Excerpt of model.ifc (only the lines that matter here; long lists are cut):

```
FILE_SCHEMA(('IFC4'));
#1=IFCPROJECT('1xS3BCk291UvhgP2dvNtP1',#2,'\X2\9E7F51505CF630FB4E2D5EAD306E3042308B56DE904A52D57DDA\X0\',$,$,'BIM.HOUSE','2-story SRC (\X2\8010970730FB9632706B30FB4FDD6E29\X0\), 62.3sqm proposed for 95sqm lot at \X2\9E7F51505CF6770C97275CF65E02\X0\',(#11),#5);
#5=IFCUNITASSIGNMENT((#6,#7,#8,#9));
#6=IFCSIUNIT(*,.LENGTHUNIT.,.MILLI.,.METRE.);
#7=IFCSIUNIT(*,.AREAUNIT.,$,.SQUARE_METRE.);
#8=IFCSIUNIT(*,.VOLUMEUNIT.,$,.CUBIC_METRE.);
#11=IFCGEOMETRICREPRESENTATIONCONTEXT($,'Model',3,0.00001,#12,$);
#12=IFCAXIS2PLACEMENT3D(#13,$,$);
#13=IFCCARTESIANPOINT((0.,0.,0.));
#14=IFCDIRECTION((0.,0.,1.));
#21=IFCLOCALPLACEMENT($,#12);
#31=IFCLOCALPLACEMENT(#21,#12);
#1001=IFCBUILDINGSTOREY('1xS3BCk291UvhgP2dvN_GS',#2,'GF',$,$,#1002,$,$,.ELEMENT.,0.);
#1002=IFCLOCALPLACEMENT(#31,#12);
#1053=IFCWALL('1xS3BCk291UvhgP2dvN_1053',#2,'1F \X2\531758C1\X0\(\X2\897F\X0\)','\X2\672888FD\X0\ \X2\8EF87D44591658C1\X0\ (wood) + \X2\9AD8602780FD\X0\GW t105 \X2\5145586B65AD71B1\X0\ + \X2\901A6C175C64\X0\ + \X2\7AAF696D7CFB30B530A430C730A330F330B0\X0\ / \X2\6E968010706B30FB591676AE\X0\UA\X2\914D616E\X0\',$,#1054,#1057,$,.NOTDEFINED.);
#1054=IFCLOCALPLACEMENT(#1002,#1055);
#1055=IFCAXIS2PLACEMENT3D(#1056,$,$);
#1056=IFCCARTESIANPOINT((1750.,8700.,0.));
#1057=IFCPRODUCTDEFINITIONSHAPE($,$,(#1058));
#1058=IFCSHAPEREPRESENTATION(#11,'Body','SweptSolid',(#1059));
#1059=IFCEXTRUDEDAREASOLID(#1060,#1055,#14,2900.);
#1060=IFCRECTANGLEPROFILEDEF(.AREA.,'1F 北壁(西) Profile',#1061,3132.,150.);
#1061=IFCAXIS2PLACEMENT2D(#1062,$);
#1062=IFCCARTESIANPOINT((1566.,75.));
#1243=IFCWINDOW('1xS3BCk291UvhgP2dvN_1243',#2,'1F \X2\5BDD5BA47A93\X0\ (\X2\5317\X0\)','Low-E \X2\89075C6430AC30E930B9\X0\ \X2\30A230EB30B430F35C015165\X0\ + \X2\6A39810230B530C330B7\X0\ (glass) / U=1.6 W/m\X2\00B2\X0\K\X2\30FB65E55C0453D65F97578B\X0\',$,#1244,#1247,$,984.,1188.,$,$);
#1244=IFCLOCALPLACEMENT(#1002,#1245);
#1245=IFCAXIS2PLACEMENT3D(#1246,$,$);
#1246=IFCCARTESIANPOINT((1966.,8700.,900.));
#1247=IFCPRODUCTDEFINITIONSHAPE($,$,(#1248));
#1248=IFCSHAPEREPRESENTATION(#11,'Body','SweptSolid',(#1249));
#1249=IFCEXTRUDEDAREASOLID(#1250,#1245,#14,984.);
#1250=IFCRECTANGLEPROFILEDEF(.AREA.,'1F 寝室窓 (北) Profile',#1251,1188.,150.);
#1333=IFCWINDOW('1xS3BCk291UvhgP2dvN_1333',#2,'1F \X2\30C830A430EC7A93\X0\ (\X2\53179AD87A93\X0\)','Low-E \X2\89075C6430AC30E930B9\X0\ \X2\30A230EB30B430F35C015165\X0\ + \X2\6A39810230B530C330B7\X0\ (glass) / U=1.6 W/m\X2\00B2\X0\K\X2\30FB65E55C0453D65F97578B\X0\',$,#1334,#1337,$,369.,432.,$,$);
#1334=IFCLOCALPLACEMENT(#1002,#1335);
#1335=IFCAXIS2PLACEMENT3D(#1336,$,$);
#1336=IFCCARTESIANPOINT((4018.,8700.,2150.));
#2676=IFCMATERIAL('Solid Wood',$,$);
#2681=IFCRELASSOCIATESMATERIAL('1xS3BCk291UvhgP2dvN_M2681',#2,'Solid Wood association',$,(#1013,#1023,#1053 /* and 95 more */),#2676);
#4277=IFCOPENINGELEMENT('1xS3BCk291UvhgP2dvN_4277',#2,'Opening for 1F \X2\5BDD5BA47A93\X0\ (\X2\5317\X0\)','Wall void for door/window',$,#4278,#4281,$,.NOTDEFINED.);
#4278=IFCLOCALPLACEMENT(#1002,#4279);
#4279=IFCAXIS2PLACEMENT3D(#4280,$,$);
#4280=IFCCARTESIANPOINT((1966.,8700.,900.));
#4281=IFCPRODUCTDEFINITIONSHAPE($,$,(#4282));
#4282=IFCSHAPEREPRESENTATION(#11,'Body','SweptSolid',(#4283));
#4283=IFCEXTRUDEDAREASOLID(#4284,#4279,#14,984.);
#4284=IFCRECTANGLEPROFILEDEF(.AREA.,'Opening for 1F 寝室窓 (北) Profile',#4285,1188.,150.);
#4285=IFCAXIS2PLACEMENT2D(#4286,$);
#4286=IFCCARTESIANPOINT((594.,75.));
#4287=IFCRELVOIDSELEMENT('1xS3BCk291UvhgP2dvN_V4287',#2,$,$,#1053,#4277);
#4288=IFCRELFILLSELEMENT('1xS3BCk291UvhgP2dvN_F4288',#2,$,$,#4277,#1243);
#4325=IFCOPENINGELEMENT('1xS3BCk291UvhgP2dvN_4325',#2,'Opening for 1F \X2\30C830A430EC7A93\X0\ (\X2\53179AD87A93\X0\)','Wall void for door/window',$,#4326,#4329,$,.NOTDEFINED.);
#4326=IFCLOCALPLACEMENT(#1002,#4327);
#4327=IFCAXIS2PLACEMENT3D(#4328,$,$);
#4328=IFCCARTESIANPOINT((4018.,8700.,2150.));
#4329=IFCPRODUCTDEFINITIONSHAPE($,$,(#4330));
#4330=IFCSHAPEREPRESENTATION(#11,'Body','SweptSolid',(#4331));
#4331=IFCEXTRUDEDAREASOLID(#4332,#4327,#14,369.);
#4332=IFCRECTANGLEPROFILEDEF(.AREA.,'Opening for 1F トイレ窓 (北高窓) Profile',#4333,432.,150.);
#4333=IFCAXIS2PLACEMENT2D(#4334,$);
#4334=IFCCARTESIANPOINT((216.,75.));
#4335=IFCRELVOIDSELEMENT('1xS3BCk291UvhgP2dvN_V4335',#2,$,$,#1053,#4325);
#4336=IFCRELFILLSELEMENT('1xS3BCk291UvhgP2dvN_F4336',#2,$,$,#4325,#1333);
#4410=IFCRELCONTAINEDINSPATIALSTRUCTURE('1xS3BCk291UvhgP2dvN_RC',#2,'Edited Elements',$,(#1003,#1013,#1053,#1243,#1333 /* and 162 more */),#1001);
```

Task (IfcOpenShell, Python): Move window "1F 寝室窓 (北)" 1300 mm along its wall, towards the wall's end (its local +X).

```python
import ifcopenshell
import ifcopenshell.api.geometry
import ifcopenshell.util.placement

model = ifcopenshell.open("model.ifc")

window = model.by_guid("1xS3BCk291UvhgP2dvN_1243")
opening = window.FillsVoids[0].RelatingOpeningElement
wall = opening.VoidsElements[0].RelatingBuildingElement

wall_matrix = ifcopenshell.util.placement.get_local_placement(wall.ObjectPlacement)
shift = wall_matrix[:3, 0] * 1300.0
before = ifcopenshell.util.placement.get_local_placement(window.ObjectPlacement)[:3, 3].copy()

# The window is not placed relative to its opening, so move both.
for product in (opening, window):
    matrix = ifcopenshell.util.placement.get_local_placement(product.ObjectPlacement)
    matrix[:3, 3] += shift
    ifcopenshell.api.geometry.edit_object_placement(model, product=product, matrix=matrix, is_si=False)

after = ifcopenshell.util.placement.get_local_placement(window.ObjectPlacement)[:3, 3]
print("window moved by", (after - before).round(3) + 0.0)

model.write("model_v2.ifc")
```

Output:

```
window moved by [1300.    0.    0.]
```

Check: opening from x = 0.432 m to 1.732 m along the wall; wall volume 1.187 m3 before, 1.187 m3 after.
